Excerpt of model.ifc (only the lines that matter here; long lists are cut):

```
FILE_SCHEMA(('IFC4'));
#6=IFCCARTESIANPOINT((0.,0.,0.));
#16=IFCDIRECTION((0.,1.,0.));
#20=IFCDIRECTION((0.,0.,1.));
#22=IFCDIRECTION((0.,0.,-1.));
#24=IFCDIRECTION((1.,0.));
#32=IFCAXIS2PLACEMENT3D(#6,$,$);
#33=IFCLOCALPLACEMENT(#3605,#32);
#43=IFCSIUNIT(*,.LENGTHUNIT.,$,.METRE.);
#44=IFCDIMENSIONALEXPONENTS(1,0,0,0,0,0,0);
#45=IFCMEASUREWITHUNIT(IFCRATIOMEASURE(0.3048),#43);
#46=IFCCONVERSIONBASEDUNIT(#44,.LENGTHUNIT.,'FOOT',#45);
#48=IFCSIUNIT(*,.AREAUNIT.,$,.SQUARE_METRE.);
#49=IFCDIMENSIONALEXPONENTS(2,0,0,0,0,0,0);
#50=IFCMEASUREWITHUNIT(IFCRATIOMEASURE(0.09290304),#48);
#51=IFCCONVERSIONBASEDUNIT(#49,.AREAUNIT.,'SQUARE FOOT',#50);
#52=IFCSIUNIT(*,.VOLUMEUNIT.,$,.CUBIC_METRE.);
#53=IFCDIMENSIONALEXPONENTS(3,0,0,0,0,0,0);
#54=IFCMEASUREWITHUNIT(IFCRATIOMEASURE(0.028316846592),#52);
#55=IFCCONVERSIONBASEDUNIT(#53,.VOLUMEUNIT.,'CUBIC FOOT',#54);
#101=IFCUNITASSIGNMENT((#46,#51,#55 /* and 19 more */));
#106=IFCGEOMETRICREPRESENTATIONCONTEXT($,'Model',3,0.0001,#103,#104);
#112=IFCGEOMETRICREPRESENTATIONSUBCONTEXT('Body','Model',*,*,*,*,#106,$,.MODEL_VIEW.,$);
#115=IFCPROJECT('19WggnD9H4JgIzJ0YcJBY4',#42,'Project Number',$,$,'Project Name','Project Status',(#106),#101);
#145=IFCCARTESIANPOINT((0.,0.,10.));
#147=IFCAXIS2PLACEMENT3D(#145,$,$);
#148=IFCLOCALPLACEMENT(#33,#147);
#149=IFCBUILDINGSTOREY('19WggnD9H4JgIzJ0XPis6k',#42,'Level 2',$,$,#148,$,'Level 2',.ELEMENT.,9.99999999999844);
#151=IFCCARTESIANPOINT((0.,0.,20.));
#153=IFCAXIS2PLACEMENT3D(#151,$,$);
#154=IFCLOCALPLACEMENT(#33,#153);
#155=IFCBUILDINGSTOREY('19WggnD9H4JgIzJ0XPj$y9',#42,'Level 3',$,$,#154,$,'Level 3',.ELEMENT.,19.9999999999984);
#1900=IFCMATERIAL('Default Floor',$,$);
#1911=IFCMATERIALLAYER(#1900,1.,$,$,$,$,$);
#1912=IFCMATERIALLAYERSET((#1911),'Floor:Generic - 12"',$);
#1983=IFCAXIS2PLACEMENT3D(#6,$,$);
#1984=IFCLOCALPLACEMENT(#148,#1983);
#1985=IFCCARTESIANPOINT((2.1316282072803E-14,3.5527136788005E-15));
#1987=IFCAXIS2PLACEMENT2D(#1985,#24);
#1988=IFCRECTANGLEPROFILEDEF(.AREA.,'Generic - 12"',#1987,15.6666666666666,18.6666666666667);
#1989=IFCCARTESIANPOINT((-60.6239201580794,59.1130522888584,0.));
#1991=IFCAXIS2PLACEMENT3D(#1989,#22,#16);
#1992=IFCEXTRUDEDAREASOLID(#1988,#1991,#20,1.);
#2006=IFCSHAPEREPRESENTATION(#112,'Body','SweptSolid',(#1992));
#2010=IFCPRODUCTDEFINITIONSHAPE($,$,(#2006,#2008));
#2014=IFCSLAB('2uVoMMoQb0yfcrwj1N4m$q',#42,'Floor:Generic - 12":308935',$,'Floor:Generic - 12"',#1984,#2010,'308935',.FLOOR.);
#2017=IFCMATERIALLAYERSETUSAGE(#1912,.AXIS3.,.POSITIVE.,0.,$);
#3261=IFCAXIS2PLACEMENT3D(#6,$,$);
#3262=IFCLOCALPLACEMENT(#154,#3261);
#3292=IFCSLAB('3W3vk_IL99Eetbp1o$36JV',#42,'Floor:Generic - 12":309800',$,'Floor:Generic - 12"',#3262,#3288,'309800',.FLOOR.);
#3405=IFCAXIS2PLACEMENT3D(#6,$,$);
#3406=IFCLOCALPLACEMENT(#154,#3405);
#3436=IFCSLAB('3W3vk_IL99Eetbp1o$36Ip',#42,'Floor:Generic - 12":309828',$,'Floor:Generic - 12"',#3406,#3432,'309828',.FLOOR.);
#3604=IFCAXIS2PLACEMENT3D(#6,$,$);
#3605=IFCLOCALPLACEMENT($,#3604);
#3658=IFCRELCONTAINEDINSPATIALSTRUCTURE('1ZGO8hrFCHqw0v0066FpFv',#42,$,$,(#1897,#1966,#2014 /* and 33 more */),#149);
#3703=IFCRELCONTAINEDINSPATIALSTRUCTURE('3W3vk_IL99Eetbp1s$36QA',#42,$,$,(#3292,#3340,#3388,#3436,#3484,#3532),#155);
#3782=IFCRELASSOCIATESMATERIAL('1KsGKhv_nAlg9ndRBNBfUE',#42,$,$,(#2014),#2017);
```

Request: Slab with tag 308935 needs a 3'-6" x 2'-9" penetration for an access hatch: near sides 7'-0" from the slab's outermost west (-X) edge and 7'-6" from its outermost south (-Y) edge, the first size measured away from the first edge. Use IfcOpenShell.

```python
import numpy as np
import ifcopenshell
import ifcopenshell.api.feature
import ifcopenshell.api.geometry
import ifcopenshell.api.root
import ifcopenshell.geom
import ifcopenshell.util.placement
import ifcopenshell.util.representation
import ifcopenshell.util.shape
import ifcopenshell.util.unit

model = ifcopenshell.open("model.ifc")
unit_scale = ifcopenshell.util.unit.calculate_unit_scale(model)
settings = ifcopenshell.geom.settings()


def volume(element):
    """Net volume in cubic metres, openings subtracted."""
    shape = ifcopenshell.geom.create_shape(settings, element)
    return ifcopenshell.util.shape.get_volume(shape.geometry)


slab = model.by_guid("2uVoMMoQb0yfcrwj1N4m$q")
before = volume(slab)

# Extent in the slab's own axes, in metres. The edges named are its -X and -Y sides.
slab_shape = ifcopenshell.geom.create_shape(settings, slab)
vertices = ifcopenshell.util.shape.get_vertices(slab_shape.geometry)
x_min, y_min, bottom = vertices.min(axis=0)
top = vertices[:, 2].max()

opening = ifcopenshell.api.root.create_entity(model, ifc_class="IfcOpeningElement", name="Access hatch opening", predefined_type="OPENING")
context = ifcopenshell.util.representation.get_context(model, "Model", "Body", "MODEL_VIEW")
width, depth = 1.0668, 0.8382
outline = [(0.0, 0.0), (width, 0.0), (width, depth), (0.0, depth), (0.0, 0.0)]
# Overshoot both faces by 50 mm so the cut is clean.
shape = ifcopenshell.api.geometry.add_slab_representation(
    model, context=context, depth=top - bottom + 0.1, polyline=outline
)
ifcopenshell.api.geometry.assign_representation(model, product=opening, representation=shape)

matrix = ifcopenshell.util.placement.get_local_placement(slab.ObjectPlacement)
matrix[:, 3] = matrix @ np.append(np.array([x_min + 2.1336, y_min + 2.286, bottom - 0.05]) / unit_scale, 1.0)
ifcopenshell.api.geometry.edit_object_placement(model, product=opening, matrix=matrix, is_si=False)
ifcopenshell.api.feature.add_feature(model, feature=opening, element=slab)

after = volume(slab)

print(f"slab volume {before:.3f} -> {after:.3f} m3")

model.write("model_rev.ifc")
```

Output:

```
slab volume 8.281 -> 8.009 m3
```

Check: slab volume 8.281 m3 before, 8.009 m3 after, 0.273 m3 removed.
